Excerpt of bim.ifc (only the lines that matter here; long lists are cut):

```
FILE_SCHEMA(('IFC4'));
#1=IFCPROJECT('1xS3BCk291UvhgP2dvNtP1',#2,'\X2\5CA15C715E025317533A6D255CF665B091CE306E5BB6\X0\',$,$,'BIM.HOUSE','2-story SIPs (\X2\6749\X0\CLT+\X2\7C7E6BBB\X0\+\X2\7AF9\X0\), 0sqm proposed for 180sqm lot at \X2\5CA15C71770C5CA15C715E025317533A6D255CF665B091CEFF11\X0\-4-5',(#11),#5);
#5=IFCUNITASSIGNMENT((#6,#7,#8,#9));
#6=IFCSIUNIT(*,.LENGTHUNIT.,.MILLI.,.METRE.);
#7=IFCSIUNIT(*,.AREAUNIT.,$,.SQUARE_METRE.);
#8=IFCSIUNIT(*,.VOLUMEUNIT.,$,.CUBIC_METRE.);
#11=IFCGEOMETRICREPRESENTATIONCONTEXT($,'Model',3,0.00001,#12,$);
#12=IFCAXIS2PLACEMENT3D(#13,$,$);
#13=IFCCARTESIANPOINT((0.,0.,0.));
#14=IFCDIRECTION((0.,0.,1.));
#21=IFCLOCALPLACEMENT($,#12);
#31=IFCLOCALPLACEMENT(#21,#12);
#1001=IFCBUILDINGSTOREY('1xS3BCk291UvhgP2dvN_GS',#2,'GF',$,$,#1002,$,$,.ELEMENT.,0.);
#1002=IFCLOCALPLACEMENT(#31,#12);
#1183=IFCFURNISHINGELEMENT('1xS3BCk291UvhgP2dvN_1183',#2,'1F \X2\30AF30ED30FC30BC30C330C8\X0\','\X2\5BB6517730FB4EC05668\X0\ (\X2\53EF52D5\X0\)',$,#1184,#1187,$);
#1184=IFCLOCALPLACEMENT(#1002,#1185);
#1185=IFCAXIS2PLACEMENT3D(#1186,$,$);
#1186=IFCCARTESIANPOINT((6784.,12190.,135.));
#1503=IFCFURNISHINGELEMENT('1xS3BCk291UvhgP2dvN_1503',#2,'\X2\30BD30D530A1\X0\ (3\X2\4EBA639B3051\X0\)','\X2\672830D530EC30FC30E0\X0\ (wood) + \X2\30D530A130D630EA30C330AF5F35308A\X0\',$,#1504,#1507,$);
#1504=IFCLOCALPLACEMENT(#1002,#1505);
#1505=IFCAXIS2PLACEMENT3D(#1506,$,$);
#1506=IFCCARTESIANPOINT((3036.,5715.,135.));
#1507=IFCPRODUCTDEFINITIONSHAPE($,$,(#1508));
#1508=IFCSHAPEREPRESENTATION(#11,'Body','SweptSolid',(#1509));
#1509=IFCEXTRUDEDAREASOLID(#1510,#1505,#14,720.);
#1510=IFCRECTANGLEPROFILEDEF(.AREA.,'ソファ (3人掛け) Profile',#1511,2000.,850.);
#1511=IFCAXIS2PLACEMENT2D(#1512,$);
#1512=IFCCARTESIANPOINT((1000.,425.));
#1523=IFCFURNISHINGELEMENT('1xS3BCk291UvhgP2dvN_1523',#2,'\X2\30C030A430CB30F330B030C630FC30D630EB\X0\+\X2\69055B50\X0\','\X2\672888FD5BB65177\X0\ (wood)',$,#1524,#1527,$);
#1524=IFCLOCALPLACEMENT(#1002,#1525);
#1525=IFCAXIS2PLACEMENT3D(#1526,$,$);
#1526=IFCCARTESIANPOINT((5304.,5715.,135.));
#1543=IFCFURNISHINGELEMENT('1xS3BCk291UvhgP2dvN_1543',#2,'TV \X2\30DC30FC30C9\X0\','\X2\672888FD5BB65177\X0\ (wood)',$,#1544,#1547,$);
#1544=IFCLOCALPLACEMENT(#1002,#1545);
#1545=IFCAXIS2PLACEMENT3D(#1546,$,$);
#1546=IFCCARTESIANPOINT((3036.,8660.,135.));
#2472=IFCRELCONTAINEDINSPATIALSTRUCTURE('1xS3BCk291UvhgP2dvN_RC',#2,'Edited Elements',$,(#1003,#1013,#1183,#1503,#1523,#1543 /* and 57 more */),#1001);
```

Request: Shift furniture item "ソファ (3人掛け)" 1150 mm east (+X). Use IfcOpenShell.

```python
import ifcopenshell
import ifcopenshell.api.geometry
import ifcopenshell.util.placement

model = ifcopenshell.open("bim.ifc")

item = model.by_id(1503)
matrix = ifcopenshell.util.placement.get_local_placement(item.ObjectPlacement)
matrix[0, 3] += 1150.0
ifcopenshell.api.geometry.edit_object_placement(model, product=item, matrix=matrix, is_si=False)

print(ifcopenshell.util.placement.get_local_placement(item.ObjectPlacement).round(3) + 0.0)

model.write("bim_rev.ifc")
```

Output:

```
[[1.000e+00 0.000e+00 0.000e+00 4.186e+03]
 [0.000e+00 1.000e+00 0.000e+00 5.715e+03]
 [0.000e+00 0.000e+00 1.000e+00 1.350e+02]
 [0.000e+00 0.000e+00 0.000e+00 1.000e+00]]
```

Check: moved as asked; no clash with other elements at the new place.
